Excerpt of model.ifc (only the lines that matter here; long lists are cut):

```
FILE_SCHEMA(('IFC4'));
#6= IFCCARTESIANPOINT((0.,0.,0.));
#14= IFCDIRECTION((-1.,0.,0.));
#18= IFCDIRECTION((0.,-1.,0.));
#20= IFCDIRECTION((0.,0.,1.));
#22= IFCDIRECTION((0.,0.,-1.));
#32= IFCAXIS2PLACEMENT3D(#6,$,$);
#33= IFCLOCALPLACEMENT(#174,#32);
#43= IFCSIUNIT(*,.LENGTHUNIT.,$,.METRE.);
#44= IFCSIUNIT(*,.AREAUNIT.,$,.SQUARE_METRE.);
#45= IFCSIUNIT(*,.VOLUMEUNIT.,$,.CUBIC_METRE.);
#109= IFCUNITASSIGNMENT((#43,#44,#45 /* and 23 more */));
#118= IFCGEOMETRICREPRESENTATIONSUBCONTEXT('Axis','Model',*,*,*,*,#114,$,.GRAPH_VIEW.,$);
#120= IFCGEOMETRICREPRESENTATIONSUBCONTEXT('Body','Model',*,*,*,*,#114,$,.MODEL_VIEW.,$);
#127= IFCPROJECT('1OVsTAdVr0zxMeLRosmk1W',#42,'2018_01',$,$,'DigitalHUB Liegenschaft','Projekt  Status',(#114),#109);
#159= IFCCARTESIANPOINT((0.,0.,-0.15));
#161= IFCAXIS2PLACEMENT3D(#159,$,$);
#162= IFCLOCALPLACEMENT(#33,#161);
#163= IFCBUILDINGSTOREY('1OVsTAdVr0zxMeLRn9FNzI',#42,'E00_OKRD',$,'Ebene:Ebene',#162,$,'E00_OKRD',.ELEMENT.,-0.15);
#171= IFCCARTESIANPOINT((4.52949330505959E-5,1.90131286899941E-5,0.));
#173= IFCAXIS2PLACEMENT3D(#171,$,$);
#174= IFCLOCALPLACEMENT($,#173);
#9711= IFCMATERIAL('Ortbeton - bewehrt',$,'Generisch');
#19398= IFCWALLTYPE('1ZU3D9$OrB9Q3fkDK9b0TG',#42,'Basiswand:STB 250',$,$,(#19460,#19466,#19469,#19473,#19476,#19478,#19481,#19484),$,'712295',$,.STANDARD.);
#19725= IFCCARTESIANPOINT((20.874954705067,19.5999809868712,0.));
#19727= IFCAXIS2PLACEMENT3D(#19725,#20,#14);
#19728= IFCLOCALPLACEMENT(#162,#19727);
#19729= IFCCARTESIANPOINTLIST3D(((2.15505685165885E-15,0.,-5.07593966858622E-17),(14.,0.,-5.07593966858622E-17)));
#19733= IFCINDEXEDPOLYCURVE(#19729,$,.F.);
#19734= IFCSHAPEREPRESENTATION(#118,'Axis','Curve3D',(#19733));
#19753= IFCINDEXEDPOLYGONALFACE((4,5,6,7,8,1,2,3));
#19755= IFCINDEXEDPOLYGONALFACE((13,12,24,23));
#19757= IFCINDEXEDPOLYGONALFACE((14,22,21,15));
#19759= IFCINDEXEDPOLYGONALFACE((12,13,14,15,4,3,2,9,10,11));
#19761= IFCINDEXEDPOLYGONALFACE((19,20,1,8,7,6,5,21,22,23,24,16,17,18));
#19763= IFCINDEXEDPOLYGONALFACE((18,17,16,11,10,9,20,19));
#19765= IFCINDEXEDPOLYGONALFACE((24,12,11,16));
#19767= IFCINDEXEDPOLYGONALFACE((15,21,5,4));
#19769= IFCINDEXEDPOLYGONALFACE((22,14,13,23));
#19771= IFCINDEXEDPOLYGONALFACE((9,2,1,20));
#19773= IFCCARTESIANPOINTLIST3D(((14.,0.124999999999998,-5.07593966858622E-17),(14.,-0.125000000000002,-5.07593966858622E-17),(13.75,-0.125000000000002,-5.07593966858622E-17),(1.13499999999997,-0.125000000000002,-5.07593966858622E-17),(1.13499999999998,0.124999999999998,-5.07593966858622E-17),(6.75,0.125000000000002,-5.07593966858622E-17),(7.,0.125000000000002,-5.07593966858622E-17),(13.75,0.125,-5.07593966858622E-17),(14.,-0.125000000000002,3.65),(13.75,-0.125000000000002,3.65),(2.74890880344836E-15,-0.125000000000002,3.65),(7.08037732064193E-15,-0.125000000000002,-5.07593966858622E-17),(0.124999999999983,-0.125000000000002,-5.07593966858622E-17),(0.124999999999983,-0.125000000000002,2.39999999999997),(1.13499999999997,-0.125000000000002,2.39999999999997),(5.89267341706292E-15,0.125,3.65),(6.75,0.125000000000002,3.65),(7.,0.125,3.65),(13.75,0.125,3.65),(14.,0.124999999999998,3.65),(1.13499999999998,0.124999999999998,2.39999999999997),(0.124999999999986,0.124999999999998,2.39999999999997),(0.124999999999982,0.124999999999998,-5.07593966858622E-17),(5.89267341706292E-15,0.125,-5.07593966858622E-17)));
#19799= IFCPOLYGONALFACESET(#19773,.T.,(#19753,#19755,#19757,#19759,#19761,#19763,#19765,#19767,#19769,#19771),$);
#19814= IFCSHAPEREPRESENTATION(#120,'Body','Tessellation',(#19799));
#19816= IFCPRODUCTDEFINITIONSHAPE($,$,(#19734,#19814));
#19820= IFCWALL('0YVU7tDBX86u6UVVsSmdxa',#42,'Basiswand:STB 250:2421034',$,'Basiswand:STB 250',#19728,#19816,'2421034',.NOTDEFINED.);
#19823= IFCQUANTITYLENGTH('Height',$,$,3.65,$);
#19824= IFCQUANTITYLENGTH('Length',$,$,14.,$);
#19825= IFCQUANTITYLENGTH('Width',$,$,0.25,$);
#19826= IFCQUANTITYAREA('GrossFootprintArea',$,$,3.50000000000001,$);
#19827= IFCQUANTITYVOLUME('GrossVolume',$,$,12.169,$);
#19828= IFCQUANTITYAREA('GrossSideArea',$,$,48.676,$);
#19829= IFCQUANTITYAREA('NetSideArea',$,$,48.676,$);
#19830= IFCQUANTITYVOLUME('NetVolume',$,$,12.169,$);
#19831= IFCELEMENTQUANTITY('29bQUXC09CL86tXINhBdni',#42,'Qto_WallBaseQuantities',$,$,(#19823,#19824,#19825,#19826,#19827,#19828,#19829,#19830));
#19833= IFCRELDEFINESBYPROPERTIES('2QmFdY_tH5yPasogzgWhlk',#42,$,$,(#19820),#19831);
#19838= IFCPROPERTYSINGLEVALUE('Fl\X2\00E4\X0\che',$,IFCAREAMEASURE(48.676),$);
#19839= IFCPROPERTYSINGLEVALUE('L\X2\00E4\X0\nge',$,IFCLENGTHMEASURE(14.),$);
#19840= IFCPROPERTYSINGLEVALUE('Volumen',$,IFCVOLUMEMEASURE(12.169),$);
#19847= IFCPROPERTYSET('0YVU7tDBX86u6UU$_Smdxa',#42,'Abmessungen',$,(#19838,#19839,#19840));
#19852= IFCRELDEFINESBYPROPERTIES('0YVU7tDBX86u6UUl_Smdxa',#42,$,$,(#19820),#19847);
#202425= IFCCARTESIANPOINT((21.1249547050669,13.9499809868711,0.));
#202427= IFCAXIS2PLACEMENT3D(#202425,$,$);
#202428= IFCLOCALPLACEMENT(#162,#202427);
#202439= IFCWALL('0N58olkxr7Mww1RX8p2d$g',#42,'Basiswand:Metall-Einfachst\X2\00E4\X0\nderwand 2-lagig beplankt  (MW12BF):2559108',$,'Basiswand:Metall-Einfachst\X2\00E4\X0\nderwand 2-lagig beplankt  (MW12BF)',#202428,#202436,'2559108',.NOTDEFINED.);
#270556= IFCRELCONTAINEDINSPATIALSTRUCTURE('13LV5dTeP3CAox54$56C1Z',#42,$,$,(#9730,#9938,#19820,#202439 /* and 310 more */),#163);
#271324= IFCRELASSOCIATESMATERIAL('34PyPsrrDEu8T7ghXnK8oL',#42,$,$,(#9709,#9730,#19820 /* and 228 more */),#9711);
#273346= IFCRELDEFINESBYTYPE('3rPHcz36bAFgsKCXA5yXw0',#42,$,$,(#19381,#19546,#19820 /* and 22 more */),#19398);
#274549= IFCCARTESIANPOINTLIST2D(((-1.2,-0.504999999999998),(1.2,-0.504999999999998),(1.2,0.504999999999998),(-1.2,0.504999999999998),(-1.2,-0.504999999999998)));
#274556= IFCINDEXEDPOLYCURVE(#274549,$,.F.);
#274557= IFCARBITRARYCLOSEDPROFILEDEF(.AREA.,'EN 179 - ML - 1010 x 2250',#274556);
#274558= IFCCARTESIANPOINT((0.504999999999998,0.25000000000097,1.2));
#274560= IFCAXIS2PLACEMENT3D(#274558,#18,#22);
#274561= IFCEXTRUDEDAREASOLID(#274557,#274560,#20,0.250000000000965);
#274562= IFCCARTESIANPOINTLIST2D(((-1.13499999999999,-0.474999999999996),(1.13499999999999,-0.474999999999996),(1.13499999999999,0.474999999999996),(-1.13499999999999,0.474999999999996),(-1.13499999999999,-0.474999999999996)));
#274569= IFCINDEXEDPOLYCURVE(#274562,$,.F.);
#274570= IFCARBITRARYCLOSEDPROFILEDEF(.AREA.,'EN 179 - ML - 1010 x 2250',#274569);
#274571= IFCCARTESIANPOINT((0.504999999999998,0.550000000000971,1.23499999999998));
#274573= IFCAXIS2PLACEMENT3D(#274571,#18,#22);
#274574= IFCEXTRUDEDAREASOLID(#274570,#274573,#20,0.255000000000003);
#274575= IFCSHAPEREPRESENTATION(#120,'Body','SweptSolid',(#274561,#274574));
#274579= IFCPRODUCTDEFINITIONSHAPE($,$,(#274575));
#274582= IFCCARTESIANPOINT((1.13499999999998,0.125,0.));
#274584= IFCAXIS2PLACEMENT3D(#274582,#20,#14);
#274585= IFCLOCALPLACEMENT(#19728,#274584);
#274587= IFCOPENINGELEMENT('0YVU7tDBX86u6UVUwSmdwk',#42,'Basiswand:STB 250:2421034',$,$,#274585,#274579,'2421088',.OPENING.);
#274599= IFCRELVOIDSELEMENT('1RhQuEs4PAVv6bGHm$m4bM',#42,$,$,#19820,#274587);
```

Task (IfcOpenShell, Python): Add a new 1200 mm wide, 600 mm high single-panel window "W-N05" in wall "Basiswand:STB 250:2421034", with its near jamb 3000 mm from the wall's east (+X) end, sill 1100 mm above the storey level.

```python
import numpy as np
import ifcopenshell
import ifcopenshell.api.feature
import ifcopenshell.api.geometry
import ifcopenshell.api.pset
import ifcopenshell.api.root
import ifcopenshell.api.spatial
import ifcopenshell.geom
import ifcopenshell.util.element
import ifcopenshell.util.placement
import ifcopenshell.util.representation
import ifcopenshell.util.shape
import ifcopenshell.util.unit

model = ifcopenshell.open("model.ifc")
unit_scale = ifcopenshell.util.unit.calculate_unit_scale(model)
area_scale = ifcopenshell.util.unit.calculate_unit_scale(model, "AREAUNIT")
volume_scale = ifcopenshell.util.unit.calculate_unit_scale(model, "VOLUMEUNIT")
settings = ifcopenshell.geom.settings()


def volume(element):
    """Net volume in cubic metres, openings subtracted."""
    shape = ifcopenshell.geom.create_shape(settings, element)
    return ifcopenshell.util.shape.get_volume(shape.geometry)


wall = model.by_guid("0YVU7tDBX86u6UVVsSmdxa")
storey = ifcopenshell.util.element.get_container(wall, ifc_class="IfcBuildingStorey")
context = ifcopenshell.util.representation.get_context(model, "Model", "Body", "MODEL_VIEW")
before = volume(wall)

width, height, from_end, sill = 1.2, 0.6, 3, 1.1  # metres

# The wall runs along its own X axis, and the end named is its -X end.
wall_shape = ifcopenshell.geom.create_shape(settings, wall)
x, y, z = ifcopenshell.util.shape.get_vertices(wall_shape.geometry).T
start = x.min() + from_end
face, thickness = float(y.min()), float(y.max() - y.min())
wall_matrix = ifcopenshell.util.placement.get_local_placement(wall.ObjectPlacement)
level = ifcopenshell.util.placement.get_local_placement(storey.ObjectPlacement)[2, 3]


def in_wall(x, y):
    """Placement at x, y metres in the wall's axes, at sill height."""
    matrix = wall_matrix.copy()
    matrix[:, 3] = wall_matrix @ np.array([x / unit_scale, y / unit_scale, 0.0, 1.0])
    matrix[2, 3] = level + sill / unit_scale
    return matrix


# Opening: a box that overshoots both wall faces by 50 mm.
opening = ifcopenshell.api.root.create_entity(model, ifc_class="IfcOpeningElement", predefined_type="OPENING")
box = ifcopenshell.api.geometry.add_wall_representation(
    model, context=context, length=width, height=height, thickness=thickness + 0.1
)
ifcopenshell.api.geometry.assign_representation(model, product=opening, representation=box)
ifcopenshell.api.geometry.edit_object_placement(model, product=opening, matrix=in_wall(start, face - 0.05), is_si=False)
ifcopenshell.api.feature.add_feature(model, feature=opening, element=wall)

window = ifcopenshell.api.root.create_entity(model, ifc_class="IfcWindow", name="W-N05", predefined_type="WINDOW")
window.OverallWidth, window.OverallHeight = width / unit_scale, height / unit_scale
window.PartitioningType = "SINGLE_PANEL"
body = ifcopenshell.api.geometry.add_window_representation(
    model,
    context=context,
    overall_width=window.OverallWidth,
    overall_height=window.OverallHeight,
    partition_type="SINGLE_PANEL",
)
ifcopenshell.api.geometry.assign_representation(model, product=window, representation=body)
ifcopenshell.api.spatial.assign_container(model, products=[window], relating_structure=storey)
ifcopenshell.api.feature.add_filling(model, opening=opening, element=window)

# Centre the window in the wall's thickness.
ifcopenshell.api.geometry.edit_object_placement(model, product=window, matrix=in_wall(start, face), is_si=False)
window_shape = ifcopenshell.geom.create_shape(settings, window)
depth = ifcopenshell.util.shape.get_vertices(window_shape.geometry)[:, 1]
offset = face + thickness / 2 - (depth.min() + depth.max()) / 2
ifcopenshell.api.geometry.edit_object_placement(model, product=window, matrix=in_wall(start, offset), is_si=False)

after = volume(wall)

# Update the wall's stored quantities.
qto = model.by_id(ifcopenshell.util.element.get_pset(wall, "Qto_WallBaseQuantities", should_inherit=False)["id"])
ifcopenshell.api.pset.edit_qto(model, qto=qto, properties={
    "NetSideArea": after / thickness / area_scale,
    "NetVolume": after / volume_scale,
})
pset = model.by_id(ifcopenshell.util.element.get_pset(wall, "Abmessungen", should_inherit=False)["id"])
ifcopenshell.api.pset.edit_pset(model, pset=pset, properties={
    "Fläche": model.create_entity("IfcAreaMeasure", after / thickness / area_scale),
    "Volumen": model.create_entity("IfcVolumeMeasure", after / volume_scale),
})

print(f"wall volume {before:.3f} -> {after:.3f} m3")

model.write("model_updated.ifc")
```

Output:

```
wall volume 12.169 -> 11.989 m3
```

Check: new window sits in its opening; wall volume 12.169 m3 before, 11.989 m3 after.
